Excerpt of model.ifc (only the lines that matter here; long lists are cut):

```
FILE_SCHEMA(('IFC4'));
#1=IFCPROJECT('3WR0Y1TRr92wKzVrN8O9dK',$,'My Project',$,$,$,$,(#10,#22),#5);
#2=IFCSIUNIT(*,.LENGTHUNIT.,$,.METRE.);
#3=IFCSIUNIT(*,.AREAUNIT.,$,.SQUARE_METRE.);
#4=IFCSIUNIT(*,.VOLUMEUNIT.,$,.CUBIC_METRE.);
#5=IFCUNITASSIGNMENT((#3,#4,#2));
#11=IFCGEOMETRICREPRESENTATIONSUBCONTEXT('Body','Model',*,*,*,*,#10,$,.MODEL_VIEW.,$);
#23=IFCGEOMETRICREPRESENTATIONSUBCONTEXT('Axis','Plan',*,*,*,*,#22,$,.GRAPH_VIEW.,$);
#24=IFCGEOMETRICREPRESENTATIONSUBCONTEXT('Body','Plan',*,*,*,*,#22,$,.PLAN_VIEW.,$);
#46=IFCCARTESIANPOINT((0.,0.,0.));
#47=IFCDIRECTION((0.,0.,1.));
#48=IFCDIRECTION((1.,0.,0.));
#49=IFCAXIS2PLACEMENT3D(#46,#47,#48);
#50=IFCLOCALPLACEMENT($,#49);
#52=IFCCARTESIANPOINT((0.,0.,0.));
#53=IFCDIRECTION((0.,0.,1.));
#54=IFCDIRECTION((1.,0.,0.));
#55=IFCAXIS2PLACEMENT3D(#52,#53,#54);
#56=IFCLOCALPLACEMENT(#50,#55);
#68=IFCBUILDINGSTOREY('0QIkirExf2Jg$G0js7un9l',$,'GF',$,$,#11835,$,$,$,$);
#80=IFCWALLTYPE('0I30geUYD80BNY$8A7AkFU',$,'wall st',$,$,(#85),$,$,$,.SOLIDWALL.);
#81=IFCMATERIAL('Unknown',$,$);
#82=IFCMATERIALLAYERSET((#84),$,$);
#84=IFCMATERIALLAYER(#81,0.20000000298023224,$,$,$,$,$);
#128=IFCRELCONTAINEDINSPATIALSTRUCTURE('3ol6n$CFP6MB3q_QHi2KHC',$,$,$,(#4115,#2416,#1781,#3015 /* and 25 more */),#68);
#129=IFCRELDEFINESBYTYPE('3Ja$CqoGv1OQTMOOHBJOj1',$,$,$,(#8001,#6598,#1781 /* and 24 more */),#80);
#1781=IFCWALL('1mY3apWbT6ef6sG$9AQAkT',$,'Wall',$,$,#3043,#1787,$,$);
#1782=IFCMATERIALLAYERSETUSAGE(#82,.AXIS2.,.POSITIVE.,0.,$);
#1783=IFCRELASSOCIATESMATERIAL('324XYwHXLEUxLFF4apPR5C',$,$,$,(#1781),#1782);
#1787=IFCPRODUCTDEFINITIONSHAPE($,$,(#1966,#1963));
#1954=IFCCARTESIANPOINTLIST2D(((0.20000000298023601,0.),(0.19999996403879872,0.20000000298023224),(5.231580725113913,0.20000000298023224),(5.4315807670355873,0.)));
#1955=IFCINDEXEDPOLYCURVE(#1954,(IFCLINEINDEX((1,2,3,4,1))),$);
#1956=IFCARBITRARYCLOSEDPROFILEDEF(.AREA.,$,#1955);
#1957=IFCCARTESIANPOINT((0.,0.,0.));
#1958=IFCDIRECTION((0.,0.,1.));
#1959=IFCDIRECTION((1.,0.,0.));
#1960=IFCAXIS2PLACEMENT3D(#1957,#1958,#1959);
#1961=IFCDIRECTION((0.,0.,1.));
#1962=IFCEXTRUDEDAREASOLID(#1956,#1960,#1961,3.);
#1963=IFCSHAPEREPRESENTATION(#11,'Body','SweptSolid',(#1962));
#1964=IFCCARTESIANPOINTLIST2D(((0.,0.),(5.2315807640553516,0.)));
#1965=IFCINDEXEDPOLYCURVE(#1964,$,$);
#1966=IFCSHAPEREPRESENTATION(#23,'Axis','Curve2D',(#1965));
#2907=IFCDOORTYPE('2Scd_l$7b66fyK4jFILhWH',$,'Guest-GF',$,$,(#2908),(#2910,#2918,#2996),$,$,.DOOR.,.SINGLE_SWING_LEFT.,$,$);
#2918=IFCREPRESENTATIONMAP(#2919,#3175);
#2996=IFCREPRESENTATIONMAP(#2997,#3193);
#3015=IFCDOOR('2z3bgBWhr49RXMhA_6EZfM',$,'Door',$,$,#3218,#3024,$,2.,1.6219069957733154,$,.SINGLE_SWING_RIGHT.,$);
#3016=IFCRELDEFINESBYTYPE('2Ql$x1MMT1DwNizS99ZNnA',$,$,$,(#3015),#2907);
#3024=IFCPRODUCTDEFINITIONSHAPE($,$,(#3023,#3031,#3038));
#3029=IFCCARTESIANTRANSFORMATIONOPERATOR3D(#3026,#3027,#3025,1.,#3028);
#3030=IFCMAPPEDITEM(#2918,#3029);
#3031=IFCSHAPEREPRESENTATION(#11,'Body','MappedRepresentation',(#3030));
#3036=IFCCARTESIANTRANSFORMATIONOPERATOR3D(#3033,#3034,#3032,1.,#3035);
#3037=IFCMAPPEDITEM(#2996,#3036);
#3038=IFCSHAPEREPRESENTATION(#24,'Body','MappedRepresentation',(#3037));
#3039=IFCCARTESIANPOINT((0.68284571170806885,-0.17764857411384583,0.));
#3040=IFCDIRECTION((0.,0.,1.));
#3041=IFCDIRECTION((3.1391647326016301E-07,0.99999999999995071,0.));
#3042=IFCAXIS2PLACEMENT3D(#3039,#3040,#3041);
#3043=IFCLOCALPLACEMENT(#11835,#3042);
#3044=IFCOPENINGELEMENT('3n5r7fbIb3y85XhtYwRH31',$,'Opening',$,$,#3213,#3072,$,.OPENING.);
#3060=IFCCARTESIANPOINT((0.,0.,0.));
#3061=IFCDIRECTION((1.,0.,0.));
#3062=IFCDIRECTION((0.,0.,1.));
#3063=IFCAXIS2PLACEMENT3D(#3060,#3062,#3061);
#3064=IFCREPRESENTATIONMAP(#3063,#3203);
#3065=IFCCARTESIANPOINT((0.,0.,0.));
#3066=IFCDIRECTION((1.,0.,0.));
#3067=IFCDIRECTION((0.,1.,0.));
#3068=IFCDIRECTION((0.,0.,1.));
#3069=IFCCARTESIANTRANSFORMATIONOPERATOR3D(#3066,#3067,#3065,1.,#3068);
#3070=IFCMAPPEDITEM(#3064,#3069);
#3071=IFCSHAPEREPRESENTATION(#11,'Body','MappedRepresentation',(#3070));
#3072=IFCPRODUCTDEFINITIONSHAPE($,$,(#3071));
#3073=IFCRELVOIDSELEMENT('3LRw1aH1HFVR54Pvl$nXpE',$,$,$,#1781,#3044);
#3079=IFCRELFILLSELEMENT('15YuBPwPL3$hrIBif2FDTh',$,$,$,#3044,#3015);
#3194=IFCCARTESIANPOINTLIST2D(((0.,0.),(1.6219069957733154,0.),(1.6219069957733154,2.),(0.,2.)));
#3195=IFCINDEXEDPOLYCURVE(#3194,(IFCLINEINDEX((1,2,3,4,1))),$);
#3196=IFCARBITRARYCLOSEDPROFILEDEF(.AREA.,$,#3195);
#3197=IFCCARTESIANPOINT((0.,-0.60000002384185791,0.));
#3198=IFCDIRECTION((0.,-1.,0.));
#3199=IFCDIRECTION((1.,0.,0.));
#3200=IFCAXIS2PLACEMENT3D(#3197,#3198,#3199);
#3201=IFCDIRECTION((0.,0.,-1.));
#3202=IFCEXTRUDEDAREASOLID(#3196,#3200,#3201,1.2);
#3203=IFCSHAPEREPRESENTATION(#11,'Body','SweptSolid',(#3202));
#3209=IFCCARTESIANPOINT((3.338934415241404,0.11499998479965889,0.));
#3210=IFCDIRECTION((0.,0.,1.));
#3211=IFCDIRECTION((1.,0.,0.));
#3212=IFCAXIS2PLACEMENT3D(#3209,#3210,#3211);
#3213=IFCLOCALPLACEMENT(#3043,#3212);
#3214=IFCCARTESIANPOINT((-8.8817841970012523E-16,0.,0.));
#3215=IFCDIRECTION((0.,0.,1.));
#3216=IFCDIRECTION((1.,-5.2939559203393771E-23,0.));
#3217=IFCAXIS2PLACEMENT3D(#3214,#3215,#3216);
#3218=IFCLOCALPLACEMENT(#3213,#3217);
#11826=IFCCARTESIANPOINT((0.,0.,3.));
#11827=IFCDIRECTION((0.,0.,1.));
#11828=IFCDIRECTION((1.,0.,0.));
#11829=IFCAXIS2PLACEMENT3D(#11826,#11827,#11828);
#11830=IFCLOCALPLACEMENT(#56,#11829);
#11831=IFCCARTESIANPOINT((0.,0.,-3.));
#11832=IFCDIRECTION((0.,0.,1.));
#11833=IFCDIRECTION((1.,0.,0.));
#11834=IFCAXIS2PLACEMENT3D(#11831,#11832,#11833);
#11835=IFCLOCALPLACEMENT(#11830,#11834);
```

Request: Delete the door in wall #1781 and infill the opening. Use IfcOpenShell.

```python
import ifcopenshell
import ifcopenshell.api.feature
import ifcopenshell.api.root
import ifcopenshell.geom
import ifcopenshell.util.shape

model = ifcopenshell.open("model.ifc")
settings = ifcopenshell.geom.settings()


def volume(element):
    """Net volume in cubic metres, openings subtracted."""
    shape = ifcopenshell.geom.create_shape(settings, element)
    return ifcopenshell.util.shape.get_volume(shape.geometry)


door = model.by_id(3015)
opening = door.FillsVoids[0].RelatingOpeningElement
wall = opening.VoidsElements[0].RelatingBuildingElement
before = volume(wall)

ifcopenshell.api.root.remove_product(model, product=door)
ifcopenshell.api.feature.remove_feature(model, feature=opening)

after = volume(wall)

print(f"wall volume {before:.3f} -> {after:.3f} m3")

model.write("model_updated.ifc")
```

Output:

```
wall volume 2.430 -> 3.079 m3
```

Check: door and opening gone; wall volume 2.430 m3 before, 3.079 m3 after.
